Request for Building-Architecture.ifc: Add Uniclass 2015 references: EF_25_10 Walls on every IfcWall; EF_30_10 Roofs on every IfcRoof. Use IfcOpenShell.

First a look at what the model holds.

```python
import ifcopenshell

model = ifcopenshell.open("Building-Architecture.ifc")
print(model.schema)
print("classifications:", [c.Name for c in model.by_type("IfcClassification")])
for ifc_class in ("IfcDoor", "IfcRoof", "IfcStair", "IfcWall", "IfcWindow"):
    print(ifc_class, len(model.by_type(ifc_class)))
```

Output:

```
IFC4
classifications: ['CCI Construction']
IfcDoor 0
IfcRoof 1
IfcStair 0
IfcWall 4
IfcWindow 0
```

```python
import ifcopenshell
import ifcopenshell.api.classification

model = ifcopenshell.open("Building-Architecture.ifc")

system = ifcopenshell.api.classification.add_classification(model, classification="Uniclass 2015")

codes = {
    "IfcWall": ("EF_25_10", "Walls"),
    "IfcRoof": ("EF_30_10", "Roofs"),
}
for ifc_class, (code, name) in codes.items():
    products = model.by_type(ifc_class)
    ifcopenshell.api.classification.add_reference(
        model, products=products, classification=system, identification=code, name=name
    )
    print(code, len(products))

model.write("Building-Architecture_edited.ifc")
```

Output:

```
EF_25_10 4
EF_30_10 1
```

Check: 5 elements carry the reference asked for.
